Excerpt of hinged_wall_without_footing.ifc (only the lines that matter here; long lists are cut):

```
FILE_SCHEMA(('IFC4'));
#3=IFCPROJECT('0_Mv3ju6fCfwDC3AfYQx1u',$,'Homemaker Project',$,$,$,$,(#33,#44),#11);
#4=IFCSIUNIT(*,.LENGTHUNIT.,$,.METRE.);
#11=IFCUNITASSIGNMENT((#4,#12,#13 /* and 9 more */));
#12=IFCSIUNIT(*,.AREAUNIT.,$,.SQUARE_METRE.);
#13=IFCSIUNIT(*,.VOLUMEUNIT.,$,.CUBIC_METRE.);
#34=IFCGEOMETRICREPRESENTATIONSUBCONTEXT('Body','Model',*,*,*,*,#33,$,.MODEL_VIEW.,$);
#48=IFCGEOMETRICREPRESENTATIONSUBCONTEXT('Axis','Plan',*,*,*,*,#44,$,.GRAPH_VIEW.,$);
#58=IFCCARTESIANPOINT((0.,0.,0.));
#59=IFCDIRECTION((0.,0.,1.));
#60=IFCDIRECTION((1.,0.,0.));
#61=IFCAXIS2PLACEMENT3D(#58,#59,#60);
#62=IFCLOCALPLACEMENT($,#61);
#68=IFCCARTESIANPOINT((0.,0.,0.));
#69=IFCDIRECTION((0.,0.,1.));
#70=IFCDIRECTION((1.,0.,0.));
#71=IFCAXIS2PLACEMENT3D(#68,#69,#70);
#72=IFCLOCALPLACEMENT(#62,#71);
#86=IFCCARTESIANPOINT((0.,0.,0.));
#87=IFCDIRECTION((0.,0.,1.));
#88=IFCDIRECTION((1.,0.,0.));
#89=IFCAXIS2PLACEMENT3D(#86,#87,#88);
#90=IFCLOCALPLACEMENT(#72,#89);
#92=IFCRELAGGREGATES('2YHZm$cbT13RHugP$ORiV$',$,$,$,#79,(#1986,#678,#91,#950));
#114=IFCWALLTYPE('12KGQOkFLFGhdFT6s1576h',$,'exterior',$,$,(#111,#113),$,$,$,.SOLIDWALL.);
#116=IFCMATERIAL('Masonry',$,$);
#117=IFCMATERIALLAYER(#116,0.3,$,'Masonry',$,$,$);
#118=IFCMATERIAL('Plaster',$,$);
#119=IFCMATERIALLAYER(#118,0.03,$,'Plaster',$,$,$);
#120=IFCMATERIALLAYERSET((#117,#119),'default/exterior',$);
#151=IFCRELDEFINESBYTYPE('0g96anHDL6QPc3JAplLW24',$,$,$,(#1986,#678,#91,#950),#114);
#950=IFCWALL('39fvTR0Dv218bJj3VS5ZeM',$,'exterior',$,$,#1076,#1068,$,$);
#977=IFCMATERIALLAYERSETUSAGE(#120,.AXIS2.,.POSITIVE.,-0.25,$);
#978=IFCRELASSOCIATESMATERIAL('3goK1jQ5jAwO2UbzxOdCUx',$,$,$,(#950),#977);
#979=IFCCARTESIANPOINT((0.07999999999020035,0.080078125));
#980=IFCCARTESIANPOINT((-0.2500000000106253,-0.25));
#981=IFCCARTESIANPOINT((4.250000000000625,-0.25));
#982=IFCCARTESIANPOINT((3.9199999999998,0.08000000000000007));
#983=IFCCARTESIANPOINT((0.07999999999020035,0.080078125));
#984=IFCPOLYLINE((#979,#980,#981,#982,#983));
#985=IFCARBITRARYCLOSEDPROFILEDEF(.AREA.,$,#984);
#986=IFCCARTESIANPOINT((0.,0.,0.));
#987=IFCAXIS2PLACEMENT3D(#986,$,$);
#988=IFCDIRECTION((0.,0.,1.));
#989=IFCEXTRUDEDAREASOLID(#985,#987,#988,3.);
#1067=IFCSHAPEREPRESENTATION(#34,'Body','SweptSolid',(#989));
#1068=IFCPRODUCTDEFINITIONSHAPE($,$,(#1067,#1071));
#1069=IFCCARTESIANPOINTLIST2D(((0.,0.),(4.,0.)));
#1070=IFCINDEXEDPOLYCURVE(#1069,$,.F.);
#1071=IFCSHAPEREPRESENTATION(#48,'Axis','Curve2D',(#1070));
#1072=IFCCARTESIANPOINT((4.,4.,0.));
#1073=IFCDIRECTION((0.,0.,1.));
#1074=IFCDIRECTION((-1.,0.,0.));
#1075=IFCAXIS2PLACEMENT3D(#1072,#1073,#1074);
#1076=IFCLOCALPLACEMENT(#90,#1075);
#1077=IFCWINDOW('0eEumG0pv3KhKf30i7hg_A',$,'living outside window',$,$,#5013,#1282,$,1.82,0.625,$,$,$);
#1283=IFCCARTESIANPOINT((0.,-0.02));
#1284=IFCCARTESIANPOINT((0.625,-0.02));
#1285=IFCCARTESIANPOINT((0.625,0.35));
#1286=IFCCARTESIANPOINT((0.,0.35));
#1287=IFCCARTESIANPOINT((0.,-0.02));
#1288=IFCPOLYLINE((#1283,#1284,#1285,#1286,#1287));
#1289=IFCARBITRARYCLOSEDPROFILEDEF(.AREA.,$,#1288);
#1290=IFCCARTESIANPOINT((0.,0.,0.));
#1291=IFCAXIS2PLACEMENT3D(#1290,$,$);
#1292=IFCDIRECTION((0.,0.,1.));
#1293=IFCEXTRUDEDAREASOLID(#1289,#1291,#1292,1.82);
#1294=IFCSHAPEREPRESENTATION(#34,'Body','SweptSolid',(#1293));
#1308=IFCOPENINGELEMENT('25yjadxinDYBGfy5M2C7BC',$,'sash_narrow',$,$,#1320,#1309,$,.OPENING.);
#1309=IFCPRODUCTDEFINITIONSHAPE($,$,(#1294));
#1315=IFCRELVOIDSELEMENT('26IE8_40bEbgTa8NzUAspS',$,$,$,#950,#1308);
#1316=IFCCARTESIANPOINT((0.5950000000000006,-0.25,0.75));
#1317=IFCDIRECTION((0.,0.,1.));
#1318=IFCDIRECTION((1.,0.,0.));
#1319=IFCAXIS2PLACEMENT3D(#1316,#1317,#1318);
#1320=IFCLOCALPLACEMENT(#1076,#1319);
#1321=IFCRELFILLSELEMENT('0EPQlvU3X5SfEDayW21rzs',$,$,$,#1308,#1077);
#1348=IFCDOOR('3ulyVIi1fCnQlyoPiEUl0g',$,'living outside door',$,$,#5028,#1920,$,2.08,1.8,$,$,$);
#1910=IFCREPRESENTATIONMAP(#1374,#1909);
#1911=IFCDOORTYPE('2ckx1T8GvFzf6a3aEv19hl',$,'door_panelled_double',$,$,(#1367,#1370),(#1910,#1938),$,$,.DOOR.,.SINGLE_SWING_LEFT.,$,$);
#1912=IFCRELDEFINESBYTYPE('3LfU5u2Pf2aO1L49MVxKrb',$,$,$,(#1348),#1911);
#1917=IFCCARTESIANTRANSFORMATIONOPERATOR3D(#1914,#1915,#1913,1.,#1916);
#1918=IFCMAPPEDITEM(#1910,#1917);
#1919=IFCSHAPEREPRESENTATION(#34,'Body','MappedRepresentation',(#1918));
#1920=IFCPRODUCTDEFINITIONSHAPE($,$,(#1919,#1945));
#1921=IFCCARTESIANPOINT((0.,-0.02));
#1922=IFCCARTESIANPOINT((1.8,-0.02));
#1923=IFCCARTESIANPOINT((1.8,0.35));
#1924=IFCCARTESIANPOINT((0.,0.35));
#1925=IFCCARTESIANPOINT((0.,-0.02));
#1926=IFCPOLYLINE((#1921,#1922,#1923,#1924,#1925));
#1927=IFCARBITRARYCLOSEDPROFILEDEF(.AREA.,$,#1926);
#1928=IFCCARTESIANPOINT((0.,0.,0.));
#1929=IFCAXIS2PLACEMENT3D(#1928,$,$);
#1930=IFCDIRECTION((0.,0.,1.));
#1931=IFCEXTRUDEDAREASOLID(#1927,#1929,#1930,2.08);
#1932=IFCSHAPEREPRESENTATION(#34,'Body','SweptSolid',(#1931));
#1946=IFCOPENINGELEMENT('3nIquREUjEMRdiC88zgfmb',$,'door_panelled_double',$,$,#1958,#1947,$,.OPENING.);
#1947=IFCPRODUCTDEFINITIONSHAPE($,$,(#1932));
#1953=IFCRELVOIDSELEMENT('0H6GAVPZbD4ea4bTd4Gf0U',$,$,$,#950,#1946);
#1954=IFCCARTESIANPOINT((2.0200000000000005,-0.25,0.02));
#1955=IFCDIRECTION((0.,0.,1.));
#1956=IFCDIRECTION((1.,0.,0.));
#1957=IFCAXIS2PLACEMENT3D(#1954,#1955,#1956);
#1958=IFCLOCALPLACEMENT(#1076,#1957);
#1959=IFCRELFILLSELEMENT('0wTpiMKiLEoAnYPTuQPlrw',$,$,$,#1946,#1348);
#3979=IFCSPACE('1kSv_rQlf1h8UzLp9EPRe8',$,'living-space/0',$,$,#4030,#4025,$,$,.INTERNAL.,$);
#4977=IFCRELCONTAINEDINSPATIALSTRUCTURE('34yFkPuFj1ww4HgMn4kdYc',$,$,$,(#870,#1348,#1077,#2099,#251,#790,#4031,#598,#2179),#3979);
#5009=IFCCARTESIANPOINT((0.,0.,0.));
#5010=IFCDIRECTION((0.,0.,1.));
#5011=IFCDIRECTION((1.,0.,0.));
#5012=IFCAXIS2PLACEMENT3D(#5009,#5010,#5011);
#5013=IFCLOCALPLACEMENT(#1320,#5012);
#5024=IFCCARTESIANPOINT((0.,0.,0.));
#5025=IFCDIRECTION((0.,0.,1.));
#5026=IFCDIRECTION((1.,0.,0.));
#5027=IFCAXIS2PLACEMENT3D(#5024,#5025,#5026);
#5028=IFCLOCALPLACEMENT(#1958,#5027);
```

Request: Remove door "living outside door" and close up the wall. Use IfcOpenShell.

```python
import ifcopenshell
import ifcopenshell.api.feature
import ifcopenshell.api.root
import ifcopenshell.geom
import ifcopenshell.util.shape

model = ifcopenshell.open("hinged_wall_without_footing.ifc")
settings = ifcopenshell.geom.settings()


def volume(element):
    """Net volume in cubic metres, openings subtracted."""
    shape = ifcopenshell.geom.create_shape(settings, element)
    return ifcopenshell.util.shape.get_volume(shape.geometry)


door = model.by_id(1348)
opening = door.FillsVoids[0].RelatingOpeningElement
wall = opening.VoidsElements[0].RelatingBuildingElement
before = volume(wall)

ifcopenshell.api.root.remove_product(model, product=door)
ifcopenshell.api.feature.remove_feature(model, feature=opening)

after = volume(wall)

print(f"wall volume {before:.3f} -> {after:.3f} m3")

model.write("hinged_wall_without_footing_v2.ifc")
```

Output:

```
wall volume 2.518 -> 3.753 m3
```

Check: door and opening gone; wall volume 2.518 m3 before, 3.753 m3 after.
